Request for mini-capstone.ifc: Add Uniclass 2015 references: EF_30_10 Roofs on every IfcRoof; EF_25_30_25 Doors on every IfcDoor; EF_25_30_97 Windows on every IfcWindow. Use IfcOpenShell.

First a look at what the model holds.

```python
import ifcopenshell

model = ifcopenshell.open("mini-capstone.ifc")
print(model.schema)
print("classifications:", [c.Name for c in model.by_type("IfcClassification")])
for ifc_class in ("IfcDoor", "IfcRoof", "IfcStair", "IfcWall", "IfcWindow"):
    print(ifc_class, len(model.by_type(ifc_class)))
```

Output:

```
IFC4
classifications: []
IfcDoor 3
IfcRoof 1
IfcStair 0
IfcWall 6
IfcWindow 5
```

```python
import ifcopenshell
import ifcopenshell.api.classification

model = ifcopenshell.open("mini-capstone.ifc")

system = ifcopenshell.api.classification.add_classification(model, classification="Uniclass 2015")

codes = {
    "IfcRoof": ("EF_30_10", "Roofs"),
    "IfcDoor": ("EF_25_30_25", "Doors"),
    "IfcWindow": ("EF_25_30_97", "Windows"),
}
for ifc_class, (code, name) in codes.items():
    products = model.by_type(ifc_class)
    ifcopenshell.api.classification.add_reference(
        model, products=products, classification=system, identification=code, name=name
    )
    print(code, len(products))

model.write("mini-capstone-out.ifc")
```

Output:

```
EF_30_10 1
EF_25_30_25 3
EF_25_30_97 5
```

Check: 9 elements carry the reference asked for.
